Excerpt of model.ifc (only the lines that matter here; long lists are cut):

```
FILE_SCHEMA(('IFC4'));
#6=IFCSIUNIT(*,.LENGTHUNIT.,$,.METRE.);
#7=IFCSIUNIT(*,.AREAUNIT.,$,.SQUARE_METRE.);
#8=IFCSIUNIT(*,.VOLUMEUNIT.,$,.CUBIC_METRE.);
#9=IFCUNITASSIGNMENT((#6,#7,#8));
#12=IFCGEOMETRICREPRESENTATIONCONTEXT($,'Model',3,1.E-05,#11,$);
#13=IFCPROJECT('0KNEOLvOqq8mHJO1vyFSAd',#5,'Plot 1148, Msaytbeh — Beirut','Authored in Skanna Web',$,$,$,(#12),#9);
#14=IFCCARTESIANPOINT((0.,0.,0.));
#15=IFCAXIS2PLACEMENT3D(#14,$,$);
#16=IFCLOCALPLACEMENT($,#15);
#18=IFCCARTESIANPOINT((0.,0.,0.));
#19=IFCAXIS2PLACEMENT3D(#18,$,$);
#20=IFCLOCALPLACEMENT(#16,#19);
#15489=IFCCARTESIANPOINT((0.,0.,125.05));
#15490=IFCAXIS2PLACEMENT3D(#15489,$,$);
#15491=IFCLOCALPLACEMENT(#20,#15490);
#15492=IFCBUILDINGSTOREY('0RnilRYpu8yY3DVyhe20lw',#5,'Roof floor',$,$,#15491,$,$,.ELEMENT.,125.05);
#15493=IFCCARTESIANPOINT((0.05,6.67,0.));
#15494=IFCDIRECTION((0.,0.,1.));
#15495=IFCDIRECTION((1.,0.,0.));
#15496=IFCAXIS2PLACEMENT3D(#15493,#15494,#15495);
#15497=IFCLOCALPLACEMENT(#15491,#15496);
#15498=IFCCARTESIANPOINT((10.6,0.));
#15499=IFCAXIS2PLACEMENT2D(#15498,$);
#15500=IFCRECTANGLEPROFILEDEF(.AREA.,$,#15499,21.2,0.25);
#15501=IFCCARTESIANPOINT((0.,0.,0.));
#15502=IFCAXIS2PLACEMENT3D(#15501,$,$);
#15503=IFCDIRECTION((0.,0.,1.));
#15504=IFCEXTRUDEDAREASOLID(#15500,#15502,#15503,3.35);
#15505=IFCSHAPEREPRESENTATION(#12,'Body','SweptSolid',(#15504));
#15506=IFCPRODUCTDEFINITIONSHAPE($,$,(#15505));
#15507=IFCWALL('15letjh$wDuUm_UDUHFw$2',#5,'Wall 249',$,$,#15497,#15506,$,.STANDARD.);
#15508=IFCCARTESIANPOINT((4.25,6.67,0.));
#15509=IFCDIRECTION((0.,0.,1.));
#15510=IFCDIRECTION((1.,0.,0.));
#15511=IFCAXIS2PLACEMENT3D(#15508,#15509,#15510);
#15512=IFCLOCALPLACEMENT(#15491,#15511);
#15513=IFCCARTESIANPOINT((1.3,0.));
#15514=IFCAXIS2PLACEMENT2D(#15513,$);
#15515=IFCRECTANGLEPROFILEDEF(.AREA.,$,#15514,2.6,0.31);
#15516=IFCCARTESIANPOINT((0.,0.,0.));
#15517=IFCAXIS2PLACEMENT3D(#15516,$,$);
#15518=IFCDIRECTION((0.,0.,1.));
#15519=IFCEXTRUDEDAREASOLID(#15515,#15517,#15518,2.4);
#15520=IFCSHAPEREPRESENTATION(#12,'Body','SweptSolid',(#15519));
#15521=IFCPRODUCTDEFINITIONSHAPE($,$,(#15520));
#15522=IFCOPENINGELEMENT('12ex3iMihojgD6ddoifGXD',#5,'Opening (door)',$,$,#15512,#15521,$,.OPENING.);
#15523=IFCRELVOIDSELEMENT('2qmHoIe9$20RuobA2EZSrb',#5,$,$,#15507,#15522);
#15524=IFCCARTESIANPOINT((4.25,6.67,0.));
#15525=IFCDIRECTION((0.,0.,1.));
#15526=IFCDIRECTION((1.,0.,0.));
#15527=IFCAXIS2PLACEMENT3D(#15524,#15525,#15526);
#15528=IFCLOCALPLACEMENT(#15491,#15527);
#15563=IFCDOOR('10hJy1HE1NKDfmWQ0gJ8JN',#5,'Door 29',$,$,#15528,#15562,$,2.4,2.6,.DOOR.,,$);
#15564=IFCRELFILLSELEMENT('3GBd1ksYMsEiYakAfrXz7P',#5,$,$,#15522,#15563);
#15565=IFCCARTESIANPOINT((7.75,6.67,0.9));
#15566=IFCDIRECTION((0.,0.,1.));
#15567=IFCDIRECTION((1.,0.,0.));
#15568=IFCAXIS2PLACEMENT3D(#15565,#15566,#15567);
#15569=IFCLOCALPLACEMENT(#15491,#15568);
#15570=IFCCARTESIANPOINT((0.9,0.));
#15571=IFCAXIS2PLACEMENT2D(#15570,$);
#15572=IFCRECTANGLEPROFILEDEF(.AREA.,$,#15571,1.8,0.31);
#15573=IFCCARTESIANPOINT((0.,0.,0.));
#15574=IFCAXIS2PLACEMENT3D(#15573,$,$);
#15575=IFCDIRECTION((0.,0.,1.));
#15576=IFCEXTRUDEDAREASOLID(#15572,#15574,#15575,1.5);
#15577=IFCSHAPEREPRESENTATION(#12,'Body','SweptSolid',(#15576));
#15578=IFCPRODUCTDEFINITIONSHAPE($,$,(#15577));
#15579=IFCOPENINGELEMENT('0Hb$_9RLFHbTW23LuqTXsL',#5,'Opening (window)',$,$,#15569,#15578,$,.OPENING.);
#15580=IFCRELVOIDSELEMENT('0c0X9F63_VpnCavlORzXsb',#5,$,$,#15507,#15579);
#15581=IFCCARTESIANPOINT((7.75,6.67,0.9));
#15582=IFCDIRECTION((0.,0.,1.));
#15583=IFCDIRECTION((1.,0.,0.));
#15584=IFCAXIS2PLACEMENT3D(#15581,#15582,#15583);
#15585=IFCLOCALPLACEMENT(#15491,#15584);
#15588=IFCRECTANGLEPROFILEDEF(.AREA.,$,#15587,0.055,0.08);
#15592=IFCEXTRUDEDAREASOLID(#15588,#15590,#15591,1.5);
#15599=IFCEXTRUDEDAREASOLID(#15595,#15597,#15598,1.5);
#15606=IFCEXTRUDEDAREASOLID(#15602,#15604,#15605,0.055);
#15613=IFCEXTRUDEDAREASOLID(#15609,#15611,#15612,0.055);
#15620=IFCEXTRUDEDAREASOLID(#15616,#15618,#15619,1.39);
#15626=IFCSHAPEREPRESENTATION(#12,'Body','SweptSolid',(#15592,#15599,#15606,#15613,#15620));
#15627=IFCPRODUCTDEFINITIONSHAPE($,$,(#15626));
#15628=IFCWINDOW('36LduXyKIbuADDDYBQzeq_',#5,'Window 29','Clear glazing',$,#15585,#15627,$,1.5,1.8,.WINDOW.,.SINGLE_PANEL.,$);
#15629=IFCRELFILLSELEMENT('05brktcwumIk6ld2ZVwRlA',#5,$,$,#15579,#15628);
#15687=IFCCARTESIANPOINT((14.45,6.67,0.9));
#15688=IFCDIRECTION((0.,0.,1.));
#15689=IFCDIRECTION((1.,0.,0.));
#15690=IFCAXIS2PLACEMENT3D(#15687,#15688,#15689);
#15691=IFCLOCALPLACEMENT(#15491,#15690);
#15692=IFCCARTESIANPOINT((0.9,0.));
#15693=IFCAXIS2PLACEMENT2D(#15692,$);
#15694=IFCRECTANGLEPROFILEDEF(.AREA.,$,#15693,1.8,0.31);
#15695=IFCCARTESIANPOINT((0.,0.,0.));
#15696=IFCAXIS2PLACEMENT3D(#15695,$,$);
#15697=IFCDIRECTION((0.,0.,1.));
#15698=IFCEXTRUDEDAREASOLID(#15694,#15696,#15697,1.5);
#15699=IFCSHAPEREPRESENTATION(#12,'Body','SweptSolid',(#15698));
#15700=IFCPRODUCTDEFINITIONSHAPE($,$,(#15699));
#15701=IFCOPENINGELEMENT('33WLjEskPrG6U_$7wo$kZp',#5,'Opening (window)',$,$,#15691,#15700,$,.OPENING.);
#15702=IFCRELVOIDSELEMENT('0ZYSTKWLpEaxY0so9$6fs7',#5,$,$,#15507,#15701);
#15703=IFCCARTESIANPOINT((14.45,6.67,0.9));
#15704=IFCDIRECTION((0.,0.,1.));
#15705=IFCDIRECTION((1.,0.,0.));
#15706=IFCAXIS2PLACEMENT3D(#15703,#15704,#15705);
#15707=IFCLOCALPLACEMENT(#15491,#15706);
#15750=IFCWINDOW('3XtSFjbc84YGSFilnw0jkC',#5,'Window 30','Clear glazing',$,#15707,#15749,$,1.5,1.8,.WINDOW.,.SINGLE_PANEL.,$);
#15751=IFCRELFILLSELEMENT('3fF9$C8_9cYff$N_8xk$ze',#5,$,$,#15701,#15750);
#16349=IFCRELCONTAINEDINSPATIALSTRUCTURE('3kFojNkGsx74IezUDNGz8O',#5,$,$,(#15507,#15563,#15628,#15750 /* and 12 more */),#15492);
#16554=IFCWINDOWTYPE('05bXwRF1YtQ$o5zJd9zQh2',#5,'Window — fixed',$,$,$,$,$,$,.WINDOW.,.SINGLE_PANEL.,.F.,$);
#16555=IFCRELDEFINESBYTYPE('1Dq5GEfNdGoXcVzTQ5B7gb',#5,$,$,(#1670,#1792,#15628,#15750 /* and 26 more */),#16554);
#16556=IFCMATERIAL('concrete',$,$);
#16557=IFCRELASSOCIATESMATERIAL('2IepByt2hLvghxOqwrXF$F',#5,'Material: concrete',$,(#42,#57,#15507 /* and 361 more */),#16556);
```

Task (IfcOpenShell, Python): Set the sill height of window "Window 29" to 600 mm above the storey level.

```python
import numpy as np
import ifcopenshell
import ifcopenshell.api.geometry
import ifcopenshell.geom
import ifcopenshell.util.element
import ifcopenshell.util.placement
import ifcopenshell.util.shape
import ifcopenshell.util.unit

model = ifcopenshell.open("model.ifc")
unit_scale = ifcopenshell.util.unit.calculate_unit_scale(model)

window = model.by_guid("36LduXyKIbuADDDYBQzeq_")
opening = window.FillsVoids[0].RelatingOpeningElement
storey = ifcopenshell.util.element.get_container(window, ifc_class="IfcBuildingStorey")
level = ifcopenshell.util.placement.get_local_placement(storey.ObjectPlacement)[2, 3]

# The opening's origin need not be at the sill, so measure its lowest point.
shape = ifcopenshell.geom.create_shape(ifcopenshell.geom.settings(), opening)
bottom = ifcopenshell.util.shape.get_shape_bottom_elevation(shape, shape.geometry) / unit_scale
dz = level + 0.6 / unit_scale - bottom

shift = np.array([0.0, 0.0, dz])
# The window is not placed relative to its opening, so move both.
for product in (opening, window):
    matrix = ifcopenshell.util.placement.get_local_placement(product.ObjectPlacement)
    matrix[:3, 3] += shift
    ifcopenshell.api.geometry.edit_object_placement(model, product=product, matrix=matrix, is_si=False)

print(f"moved by {dz * unit_scale:+.3f} m")

model.write("model_rev.ifc")
```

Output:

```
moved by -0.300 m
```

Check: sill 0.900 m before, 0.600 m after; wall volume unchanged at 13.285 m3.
